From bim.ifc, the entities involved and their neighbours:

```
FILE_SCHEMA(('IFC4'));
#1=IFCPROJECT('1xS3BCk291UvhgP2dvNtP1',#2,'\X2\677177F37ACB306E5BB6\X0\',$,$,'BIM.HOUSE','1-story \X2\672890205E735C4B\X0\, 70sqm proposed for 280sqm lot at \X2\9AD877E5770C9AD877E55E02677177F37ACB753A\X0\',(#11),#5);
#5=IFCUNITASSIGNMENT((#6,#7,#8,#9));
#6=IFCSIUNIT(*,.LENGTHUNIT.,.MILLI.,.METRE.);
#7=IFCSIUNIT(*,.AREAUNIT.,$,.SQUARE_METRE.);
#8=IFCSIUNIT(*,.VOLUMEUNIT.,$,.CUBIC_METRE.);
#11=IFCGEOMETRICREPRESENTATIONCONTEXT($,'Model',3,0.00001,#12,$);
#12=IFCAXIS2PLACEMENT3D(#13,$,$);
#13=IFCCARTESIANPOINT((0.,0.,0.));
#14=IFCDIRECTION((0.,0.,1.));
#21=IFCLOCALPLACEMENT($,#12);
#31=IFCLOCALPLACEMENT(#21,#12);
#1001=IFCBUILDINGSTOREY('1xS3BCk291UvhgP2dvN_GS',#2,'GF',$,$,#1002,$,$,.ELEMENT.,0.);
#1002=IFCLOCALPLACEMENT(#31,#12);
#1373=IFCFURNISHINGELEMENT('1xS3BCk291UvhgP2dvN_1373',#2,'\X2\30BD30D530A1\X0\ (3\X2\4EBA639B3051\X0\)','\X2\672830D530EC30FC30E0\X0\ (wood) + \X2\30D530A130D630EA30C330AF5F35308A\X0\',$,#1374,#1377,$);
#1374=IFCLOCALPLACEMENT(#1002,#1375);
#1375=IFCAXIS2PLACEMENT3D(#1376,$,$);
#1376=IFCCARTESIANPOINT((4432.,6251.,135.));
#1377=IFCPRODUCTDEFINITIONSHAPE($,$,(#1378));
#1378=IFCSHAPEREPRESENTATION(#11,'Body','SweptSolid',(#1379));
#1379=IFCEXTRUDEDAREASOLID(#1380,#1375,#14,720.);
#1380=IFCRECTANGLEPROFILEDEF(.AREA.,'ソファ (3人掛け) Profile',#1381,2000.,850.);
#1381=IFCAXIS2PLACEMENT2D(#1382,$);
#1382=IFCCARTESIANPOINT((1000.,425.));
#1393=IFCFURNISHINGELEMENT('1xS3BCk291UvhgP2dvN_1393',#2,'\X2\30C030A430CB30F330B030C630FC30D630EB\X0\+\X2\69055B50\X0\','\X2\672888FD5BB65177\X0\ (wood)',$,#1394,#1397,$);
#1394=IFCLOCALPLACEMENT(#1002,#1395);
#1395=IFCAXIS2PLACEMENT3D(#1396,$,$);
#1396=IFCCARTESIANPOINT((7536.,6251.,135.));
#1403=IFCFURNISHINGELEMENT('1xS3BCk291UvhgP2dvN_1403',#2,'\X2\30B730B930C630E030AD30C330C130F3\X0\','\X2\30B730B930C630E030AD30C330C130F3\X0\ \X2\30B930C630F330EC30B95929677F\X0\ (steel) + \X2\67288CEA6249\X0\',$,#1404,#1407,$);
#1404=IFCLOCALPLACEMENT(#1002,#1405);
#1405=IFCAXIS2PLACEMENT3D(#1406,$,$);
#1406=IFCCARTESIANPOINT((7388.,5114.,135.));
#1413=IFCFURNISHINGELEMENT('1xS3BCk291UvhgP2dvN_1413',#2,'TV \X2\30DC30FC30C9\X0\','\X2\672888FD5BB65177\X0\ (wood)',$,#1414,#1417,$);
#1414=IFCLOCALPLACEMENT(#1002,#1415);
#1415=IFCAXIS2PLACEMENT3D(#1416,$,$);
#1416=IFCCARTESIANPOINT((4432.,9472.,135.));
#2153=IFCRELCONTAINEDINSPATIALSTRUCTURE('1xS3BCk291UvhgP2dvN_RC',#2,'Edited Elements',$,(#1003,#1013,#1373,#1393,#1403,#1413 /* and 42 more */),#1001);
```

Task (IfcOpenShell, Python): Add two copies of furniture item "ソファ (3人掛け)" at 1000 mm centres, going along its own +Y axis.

```python
import ifcopenshell
import ifcopenshell.api.geometry
import ifcopenshell.api.root
import ifcopenshell.util.element
import ifcopenshell.util.placement
import ifcopenshell.util.unit

model = ifcopenshell.open("bim.ifc")
unit_scale = ifcopenshell.util.unit.calculate_unit_scale(model)


def reuse_history(source, copy):
    """copy_class also copies each property set's owner history, people and application; keep the originals."""
    for rel in copy.IsDefinedBy:
        if rel.is_a("IfcRelDefinesByProperties") and (history := rel.RelatingPropertyDefinition.OwnerHistory):
            rel.RelatingPropertyDefinition.OwnerHistory = source.OwnerHistory
            ifcopenshell.util.element.remove_deep2(model, history)


source = model.by_id(1373)
base = ifcopenshell.util.placement.get_local_placement(source.ObjectPlacement)
step = base[:3, 1] * 1 / unit_scale

for i in range(1, 3):
    copy = ifcopenshell.api.root.copy_class(model, product=source)
    copy.Representation = ifcopenshell.util.element.copy_deep(
        model, source.Representation, exclude=["IfcGeometricRepresentationContext", "IfcRepresentationMap"]
    )
    reuse_history(source, copy)
    matrix = base.copy()
    matrix[:3, 3] += i * step
    print("added at", matrix[:3, 3].round(3) + 0.0)
    ifcopenshell.api.geometry.edit_object_placement(model, product=copy, matrix=matrix, is_si=False)

model.write("bim_edited.ifc")
```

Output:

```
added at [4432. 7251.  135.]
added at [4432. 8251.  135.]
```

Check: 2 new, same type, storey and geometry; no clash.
